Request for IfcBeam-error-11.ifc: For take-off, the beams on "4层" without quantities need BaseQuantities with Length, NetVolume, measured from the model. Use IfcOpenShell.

First a look at what the model holds.

```python
import ifcopenshell
import ifcopenshell.util.element
import ifcopenshell.util.unit

model = ifcopenshell.open("IfcBeam-error-11.ifc")
print(model.schema)
for unit_type in ("LENGTHUNIT", "AREAUNIT", "VOLUMEUNIT"):
    print(unit_type, ifcopenshell.util.unit.calculate_unit_scale(model, unit_type))
storey = next(s for s in model.by_type("IfcBuildingStorey") if s.Name == "4层")
beams = [e for e in ifcopenshell.util.element.get_decomposition(storey) if e.is_a("IfcBeam")]
for e in sorted(beams, key=lambda e: e.id()):
    print(e.id(), e.is_a(), e.Name, list(ifcopenshell.util.element.get_psets(e, qtos_only=True)), sep=" | ")
```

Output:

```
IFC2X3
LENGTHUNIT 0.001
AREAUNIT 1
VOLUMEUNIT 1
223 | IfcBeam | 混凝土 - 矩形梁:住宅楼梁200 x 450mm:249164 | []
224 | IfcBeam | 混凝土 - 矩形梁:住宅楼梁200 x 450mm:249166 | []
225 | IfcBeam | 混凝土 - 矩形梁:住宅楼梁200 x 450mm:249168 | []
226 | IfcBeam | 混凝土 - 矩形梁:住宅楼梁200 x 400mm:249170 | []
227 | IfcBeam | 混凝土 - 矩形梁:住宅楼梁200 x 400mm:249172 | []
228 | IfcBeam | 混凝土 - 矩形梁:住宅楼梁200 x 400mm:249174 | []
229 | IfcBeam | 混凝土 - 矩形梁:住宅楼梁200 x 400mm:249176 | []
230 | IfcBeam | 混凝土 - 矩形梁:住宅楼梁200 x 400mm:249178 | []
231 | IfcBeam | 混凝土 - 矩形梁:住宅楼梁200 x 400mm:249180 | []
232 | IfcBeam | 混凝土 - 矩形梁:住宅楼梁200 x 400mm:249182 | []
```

```python
import ifcopenshell
import ifcopenshell.api.pset
import ifcopenshell.geom
import ifcopenshell.util.element
import ifcopenshell.util.shape
import ifcopenshell.util.unit

model = ifcopenshell.open("IfcBeam-error-11.ifc")
unit_scale = ifcopenshell.util.unit.calculate_unit_scale(model)
volume_scale = ifcopenshell.util.unit.calculate_unit_scale(model, "VOLUMEUNIT")
settings = ifcopenshell.geom.settings()

storey = next(s for s in model.by_type("IfcBuildingStorey") if s.Name == "4层")
beams = [e for e in ifcopenshell.util.element.get_decomposition(storey) if e.is_a("IfcBeam")]

for e in sorted(beams, key=lambda e: e.id()):
    if ifcopenshell.util.element.get_psets(e, qtos_only=True, should_inherit=False):
        continue
    # Geometry comes back in metres, in the element's own axes.
    shape = ifcopenshell.geom.create_shape(settings, e)
    values = {
        "Length": ifcopenshell.util.shape.get_max_xyz(shape.geometry) / unit_scale,
        "NetVolume": ifcopenshell.util.shape.get_volume(shape.geometry) / volume_scale,
    }
    qto = ifcopenshell.api.pset.add_qto(model, product=e, name="BaseQuantities")
    ifcopenshell.api.pset.edit_qto(model, qto=qto, properties=values)
    print(e.id(), {k: round(v, 3) for k, v in values.items()})

model.write("IfcBeam-error-11_rev.ifc")
```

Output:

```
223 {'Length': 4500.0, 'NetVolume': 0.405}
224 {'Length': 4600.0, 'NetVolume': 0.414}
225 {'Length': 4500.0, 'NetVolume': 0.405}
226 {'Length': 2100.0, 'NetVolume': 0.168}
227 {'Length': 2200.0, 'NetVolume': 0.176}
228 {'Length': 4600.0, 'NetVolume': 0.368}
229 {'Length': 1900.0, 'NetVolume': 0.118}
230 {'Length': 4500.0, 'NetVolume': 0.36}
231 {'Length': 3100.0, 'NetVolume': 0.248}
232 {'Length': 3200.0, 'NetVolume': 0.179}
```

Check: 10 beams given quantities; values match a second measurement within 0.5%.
